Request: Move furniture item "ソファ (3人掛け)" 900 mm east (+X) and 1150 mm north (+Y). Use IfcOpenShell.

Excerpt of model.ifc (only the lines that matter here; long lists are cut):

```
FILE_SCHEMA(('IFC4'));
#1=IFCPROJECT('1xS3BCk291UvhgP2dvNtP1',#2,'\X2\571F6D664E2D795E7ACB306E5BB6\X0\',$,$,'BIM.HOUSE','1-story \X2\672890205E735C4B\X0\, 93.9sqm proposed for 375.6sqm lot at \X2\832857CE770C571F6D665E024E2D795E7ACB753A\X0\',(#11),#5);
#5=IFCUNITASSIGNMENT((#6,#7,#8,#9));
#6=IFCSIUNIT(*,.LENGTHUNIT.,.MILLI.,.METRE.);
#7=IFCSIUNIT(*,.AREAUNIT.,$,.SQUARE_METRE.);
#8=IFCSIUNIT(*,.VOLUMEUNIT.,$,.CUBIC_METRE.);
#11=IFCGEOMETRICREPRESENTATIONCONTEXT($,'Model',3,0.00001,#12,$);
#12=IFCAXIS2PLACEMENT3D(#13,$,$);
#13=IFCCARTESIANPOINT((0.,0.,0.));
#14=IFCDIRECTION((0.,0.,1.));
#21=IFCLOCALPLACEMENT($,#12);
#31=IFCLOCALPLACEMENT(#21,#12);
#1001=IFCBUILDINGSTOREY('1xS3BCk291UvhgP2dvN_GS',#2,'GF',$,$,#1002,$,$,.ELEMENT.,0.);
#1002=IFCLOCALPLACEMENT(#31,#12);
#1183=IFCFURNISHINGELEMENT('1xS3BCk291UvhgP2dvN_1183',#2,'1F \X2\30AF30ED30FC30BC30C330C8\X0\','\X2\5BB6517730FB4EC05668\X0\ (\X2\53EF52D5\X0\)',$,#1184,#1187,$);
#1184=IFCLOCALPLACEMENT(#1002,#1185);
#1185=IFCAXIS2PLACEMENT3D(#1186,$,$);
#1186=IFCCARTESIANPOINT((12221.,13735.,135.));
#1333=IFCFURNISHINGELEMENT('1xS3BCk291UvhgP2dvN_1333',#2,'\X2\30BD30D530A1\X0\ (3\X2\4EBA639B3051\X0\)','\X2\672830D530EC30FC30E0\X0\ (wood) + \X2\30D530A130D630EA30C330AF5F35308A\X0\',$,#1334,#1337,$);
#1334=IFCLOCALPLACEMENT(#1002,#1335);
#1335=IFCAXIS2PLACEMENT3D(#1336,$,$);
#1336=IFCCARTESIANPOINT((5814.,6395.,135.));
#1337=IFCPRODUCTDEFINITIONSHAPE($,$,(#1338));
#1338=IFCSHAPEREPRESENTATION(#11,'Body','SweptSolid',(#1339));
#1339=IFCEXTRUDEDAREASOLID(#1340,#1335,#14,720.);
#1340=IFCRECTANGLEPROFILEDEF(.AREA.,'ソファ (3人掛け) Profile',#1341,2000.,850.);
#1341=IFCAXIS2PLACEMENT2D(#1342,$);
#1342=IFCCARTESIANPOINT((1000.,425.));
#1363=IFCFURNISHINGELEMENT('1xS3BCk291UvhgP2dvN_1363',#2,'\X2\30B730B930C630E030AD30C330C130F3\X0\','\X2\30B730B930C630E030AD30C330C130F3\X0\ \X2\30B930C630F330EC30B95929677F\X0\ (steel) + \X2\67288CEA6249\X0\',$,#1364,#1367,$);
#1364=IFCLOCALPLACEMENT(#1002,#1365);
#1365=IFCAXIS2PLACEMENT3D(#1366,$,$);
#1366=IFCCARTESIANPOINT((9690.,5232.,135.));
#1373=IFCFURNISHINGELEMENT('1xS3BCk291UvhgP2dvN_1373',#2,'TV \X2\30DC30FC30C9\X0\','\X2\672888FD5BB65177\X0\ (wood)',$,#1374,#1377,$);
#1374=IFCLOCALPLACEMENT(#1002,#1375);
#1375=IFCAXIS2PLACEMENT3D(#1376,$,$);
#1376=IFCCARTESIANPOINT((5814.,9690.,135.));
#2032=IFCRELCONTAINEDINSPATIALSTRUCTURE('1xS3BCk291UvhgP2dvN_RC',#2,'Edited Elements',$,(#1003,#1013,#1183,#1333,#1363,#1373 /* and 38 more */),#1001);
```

```python
import ifcopenshell
import ifcopenshell.api.geometry
import ifcopenshell.util.placement
import ifcopenshell.util.unit

model = ifcopenshell.open("model.ifc")
unit_scale = ifcopenshell.util.unit.calculate_unit_scale(model)

item = model.by_guid("1xS3BCk291UvhgP2dvN_1333")
matrix = ifcopenshell.util.placement.get_local_placement(item.ObjectPlacement)
matrix[0, 3] += 0.9 / unit_scale
matrix[1, 3] += 1.15 / unit_scale
ifcopenshell.api.geometry.edit_object_placement(model, product=item, matrix=matrix, is_si=False)

print(ifcopenshell.util.placement.get_local_placement(item.ObjectPlacement).round(3) + 0.0)

model.write("model_rev.ifc")
```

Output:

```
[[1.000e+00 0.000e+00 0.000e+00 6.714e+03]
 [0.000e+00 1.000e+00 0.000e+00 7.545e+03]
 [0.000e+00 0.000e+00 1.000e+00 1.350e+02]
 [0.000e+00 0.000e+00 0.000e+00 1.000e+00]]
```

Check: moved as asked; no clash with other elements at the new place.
